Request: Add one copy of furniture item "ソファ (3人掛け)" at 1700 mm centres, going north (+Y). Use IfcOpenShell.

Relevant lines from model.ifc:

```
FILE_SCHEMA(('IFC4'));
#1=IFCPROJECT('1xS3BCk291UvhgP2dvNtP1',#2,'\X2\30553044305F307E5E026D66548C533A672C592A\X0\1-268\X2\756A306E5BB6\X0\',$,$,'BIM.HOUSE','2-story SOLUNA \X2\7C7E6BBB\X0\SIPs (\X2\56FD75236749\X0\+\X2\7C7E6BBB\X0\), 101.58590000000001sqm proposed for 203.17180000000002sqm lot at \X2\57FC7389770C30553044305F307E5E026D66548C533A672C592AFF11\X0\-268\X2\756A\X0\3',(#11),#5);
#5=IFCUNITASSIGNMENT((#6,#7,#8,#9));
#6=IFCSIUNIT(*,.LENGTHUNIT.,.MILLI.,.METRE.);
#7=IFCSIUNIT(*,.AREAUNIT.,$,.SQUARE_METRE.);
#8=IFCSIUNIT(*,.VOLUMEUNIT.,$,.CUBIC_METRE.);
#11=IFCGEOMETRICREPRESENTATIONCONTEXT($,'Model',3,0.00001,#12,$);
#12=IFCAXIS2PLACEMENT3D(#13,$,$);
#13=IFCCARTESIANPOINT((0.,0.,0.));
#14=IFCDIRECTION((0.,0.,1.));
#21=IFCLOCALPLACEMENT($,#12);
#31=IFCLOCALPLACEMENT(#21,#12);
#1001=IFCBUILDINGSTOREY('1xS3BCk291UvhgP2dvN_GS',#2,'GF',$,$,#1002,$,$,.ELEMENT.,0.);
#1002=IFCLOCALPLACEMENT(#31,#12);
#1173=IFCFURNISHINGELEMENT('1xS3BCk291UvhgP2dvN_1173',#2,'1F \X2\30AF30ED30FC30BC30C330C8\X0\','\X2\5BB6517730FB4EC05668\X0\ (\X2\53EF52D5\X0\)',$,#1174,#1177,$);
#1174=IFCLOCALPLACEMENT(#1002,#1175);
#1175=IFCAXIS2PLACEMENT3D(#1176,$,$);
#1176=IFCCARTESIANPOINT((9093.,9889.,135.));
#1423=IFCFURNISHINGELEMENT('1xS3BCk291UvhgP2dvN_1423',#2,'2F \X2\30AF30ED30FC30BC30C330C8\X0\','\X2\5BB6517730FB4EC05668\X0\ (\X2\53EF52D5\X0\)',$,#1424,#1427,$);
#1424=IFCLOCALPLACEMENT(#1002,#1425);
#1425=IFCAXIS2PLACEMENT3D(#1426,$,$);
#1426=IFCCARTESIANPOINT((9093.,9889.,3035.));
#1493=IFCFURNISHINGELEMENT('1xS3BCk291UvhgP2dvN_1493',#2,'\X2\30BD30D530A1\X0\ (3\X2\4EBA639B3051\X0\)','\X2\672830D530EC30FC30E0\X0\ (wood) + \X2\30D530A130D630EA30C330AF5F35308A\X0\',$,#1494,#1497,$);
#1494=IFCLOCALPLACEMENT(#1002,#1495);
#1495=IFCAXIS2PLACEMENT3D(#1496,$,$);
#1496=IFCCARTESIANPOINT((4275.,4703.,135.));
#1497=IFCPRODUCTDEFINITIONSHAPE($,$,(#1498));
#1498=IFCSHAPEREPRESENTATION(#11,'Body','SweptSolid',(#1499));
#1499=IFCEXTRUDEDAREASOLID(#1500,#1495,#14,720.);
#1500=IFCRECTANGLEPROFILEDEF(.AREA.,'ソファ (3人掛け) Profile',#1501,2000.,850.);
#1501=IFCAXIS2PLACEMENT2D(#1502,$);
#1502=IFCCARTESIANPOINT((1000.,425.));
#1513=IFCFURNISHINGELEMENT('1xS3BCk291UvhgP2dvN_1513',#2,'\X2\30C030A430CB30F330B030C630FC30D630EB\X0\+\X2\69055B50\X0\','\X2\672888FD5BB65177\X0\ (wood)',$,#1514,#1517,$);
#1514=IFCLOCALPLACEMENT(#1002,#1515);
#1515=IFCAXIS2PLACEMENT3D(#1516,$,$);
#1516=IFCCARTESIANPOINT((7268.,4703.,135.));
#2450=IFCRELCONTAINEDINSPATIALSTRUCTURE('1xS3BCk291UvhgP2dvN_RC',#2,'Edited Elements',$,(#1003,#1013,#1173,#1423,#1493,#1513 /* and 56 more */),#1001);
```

```python
import numpy as np
import ifcopenshell
import ifcopenshell.api.geometry
import ifcopenshell.api.root
import ifcopenshell.util.element
import ifcopenshell.util.placement
import ifcopenshell.util.unit

model = ifcopenshell.open("model.ifc")
unit_scale = ifcopenshell.util.unit.calculate_unit_scale(model)


def reuse_history(source, copy):
    """copy_class also copies each property set's owner history, people and application; keep the originals."""
    for rel in copy.IsDefinedBy:
        if rel.is_a("IfcRelDefinesByProperties") and (history := rel.RelatingPropertyDefinition.OwnerHistory):
            rel.RelatingPropertyDefinition.OwnerHistory = source.OwnerHistory
            ifcopenshell.util.element.remove_deep2(model, history)


source = model.by_guid("1xS3BCk291UvhgP2dvN_1493")
base = ifcopenshell.util.placement.get_local_placement(source.ObjectPlacement)
step = np.array([0.0, 1.0, 0.0]) * 1.7 / unit_scale

for i in range(1, 2):
    copy = ifcopenshell.api.root.copy_class(model, product=source)
    copy.Representation = ifcopenshell.util.element.copy_deep(
        model, source.Representation, exclude=["IfcGeometricRepresentationContext", "IfcRepresentationMap"]
    )
    reuse_history(source, copy)
    matrix = base.copy()
    matrix[:3, 3] += i * step
    print("added at", matrix[:3, 3].round(3) + 0.0)
    ifcopenshell.api.geometry.edit_object_placement(model, product=copy, matrix=matrix, is_si=False)

model.write("model_updated.ifc")
```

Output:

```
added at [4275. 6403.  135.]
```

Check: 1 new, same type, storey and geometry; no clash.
